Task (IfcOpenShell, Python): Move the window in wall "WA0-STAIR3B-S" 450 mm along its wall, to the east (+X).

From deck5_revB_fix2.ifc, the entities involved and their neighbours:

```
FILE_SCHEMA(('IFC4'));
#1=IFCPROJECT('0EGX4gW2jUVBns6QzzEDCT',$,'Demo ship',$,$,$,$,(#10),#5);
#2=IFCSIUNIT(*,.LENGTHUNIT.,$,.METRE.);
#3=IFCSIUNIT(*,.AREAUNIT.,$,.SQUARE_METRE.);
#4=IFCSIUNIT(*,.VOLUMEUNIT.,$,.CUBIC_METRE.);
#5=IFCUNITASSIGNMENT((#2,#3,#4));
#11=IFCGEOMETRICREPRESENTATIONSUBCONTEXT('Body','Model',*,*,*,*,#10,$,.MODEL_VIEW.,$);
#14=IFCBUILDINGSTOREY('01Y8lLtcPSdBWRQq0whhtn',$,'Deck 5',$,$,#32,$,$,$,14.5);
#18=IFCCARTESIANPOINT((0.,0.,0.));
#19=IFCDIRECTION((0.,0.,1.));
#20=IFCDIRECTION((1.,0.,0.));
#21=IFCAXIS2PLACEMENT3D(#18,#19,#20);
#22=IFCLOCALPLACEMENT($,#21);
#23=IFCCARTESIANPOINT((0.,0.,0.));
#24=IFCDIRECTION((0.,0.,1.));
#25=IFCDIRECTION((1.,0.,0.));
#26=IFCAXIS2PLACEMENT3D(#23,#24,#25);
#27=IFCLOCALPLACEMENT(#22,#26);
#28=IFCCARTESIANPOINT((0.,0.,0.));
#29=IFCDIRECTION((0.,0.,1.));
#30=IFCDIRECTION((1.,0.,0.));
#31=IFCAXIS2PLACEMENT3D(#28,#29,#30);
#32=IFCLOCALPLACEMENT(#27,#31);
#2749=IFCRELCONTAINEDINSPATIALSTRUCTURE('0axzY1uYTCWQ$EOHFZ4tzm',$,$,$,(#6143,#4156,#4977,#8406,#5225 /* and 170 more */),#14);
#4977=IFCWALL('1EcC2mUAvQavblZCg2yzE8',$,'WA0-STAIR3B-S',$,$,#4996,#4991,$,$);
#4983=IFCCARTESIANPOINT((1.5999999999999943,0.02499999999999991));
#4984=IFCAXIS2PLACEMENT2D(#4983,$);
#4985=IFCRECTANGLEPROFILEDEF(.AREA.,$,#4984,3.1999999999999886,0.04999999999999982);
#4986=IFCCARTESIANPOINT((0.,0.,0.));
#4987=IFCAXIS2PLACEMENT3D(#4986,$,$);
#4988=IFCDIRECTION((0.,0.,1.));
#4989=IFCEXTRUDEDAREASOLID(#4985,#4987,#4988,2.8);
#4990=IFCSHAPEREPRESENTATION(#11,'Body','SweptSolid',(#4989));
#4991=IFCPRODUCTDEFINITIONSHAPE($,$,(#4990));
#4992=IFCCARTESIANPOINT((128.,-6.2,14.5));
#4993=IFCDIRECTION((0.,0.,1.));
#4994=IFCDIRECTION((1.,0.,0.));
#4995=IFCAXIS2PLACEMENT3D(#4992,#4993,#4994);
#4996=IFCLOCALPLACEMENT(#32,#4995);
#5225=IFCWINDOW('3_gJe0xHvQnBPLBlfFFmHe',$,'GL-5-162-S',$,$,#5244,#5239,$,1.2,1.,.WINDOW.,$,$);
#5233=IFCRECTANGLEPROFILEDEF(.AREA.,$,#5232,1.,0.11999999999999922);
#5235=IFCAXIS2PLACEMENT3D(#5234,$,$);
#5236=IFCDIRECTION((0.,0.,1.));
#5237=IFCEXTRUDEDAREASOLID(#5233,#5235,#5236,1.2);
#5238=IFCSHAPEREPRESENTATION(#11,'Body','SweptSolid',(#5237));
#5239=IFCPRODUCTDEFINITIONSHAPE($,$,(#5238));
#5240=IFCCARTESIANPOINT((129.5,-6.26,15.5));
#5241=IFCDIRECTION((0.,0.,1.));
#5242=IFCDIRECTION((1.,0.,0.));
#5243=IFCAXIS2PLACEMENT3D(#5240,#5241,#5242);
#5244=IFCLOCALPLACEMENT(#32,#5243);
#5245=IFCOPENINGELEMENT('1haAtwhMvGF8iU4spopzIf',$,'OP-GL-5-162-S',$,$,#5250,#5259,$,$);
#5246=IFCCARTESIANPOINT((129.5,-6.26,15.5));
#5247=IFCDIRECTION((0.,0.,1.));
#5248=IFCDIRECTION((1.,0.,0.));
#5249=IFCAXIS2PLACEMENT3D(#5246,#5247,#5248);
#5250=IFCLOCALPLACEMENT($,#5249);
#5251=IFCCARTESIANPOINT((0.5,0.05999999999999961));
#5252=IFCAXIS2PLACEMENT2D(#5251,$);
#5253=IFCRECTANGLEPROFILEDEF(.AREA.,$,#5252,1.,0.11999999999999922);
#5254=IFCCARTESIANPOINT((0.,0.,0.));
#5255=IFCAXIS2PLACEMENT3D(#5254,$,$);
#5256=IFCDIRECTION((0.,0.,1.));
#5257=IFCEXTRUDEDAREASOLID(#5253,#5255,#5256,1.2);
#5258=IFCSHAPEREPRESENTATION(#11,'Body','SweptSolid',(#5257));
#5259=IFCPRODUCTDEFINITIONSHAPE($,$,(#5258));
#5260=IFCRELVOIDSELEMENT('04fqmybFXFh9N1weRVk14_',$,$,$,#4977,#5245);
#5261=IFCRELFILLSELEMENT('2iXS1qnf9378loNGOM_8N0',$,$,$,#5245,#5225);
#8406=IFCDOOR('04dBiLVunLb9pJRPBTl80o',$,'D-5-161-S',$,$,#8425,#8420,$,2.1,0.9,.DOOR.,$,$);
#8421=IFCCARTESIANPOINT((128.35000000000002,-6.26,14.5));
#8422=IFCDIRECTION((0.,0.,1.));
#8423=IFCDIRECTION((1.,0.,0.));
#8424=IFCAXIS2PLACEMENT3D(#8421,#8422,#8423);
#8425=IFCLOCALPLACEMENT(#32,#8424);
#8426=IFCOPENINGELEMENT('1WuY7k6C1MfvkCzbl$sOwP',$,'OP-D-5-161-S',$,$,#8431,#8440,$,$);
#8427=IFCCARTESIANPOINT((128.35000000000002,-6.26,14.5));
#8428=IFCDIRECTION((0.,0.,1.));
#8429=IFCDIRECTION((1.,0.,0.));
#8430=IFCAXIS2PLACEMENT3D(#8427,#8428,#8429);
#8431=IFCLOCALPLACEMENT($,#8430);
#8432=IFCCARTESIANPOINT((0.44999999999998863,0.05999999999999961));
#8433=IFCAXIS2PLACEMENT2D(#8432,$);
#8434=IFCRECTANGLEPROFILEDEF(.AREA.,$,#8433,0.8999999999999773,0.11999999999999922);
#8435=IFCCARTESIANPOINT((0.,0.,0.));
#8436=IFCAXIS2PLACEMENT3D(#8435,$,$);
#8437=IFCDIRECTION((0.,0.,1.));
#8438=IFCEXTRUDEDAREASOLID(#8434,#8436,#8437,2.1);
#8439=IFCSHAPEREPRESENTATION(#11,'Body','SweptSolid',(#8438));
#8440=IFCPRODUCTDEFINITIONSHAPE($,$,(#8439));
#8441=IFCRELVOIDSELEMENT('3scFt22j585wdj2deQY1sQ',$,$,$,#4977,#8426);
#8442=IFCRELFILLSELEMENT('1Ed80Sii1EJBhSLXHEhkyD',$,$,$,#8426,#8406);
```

```python
import ifcopenshell
import ifcopenshell.api.geometry
import ifcopenshell.util.placement
import ifcopenshell.util.unit

model = ifcopenshell.open("deck5_revB_fix2.ifc")
unit_scale = ifcopenshell.util.unit.calculate_unit_scale(model)

window = model.by_guid("3_gJe0xHvQnBPLBlfFFmHe")
opening = window.FillsVoids[0].RelatingOpeningElement
wall = opening.VoidsElements[0].RelatingBuildingElement

wall_matrix = ifcopenshell.util.placement.get_local_placement(wall.ObjectPlacement)
shift = wall_matrix[:3, 0] * 0.45 / unit_scale
before = ifcopenshell.util.placement.get_local_placement(window.ObjectPlacement)[:3, 3].copy()

# The window is not placed relative to its opening, so move both.
for product in (opening, window):
    matrix = ifcopenshell.util.placement.get_local_placement(product.ObjectPlacement)
    matrix[:3, 3] += shift
    ifcopenshell.api.geometry.edit_object_placement(model, product=product, matrix=matrix, is_si=False)

after = ifcopenshell.util.placement.get_local_placement(window.ObjectPlacement)[:3, 3]
print("window moved by", (after - before).round(3) + 0.0)

model.write("deck5_revB_fix2_updated.ifc")
```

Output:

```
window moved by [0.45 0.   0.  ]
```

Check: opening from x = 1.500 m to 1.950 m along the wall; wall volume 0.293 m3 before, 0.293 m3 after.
